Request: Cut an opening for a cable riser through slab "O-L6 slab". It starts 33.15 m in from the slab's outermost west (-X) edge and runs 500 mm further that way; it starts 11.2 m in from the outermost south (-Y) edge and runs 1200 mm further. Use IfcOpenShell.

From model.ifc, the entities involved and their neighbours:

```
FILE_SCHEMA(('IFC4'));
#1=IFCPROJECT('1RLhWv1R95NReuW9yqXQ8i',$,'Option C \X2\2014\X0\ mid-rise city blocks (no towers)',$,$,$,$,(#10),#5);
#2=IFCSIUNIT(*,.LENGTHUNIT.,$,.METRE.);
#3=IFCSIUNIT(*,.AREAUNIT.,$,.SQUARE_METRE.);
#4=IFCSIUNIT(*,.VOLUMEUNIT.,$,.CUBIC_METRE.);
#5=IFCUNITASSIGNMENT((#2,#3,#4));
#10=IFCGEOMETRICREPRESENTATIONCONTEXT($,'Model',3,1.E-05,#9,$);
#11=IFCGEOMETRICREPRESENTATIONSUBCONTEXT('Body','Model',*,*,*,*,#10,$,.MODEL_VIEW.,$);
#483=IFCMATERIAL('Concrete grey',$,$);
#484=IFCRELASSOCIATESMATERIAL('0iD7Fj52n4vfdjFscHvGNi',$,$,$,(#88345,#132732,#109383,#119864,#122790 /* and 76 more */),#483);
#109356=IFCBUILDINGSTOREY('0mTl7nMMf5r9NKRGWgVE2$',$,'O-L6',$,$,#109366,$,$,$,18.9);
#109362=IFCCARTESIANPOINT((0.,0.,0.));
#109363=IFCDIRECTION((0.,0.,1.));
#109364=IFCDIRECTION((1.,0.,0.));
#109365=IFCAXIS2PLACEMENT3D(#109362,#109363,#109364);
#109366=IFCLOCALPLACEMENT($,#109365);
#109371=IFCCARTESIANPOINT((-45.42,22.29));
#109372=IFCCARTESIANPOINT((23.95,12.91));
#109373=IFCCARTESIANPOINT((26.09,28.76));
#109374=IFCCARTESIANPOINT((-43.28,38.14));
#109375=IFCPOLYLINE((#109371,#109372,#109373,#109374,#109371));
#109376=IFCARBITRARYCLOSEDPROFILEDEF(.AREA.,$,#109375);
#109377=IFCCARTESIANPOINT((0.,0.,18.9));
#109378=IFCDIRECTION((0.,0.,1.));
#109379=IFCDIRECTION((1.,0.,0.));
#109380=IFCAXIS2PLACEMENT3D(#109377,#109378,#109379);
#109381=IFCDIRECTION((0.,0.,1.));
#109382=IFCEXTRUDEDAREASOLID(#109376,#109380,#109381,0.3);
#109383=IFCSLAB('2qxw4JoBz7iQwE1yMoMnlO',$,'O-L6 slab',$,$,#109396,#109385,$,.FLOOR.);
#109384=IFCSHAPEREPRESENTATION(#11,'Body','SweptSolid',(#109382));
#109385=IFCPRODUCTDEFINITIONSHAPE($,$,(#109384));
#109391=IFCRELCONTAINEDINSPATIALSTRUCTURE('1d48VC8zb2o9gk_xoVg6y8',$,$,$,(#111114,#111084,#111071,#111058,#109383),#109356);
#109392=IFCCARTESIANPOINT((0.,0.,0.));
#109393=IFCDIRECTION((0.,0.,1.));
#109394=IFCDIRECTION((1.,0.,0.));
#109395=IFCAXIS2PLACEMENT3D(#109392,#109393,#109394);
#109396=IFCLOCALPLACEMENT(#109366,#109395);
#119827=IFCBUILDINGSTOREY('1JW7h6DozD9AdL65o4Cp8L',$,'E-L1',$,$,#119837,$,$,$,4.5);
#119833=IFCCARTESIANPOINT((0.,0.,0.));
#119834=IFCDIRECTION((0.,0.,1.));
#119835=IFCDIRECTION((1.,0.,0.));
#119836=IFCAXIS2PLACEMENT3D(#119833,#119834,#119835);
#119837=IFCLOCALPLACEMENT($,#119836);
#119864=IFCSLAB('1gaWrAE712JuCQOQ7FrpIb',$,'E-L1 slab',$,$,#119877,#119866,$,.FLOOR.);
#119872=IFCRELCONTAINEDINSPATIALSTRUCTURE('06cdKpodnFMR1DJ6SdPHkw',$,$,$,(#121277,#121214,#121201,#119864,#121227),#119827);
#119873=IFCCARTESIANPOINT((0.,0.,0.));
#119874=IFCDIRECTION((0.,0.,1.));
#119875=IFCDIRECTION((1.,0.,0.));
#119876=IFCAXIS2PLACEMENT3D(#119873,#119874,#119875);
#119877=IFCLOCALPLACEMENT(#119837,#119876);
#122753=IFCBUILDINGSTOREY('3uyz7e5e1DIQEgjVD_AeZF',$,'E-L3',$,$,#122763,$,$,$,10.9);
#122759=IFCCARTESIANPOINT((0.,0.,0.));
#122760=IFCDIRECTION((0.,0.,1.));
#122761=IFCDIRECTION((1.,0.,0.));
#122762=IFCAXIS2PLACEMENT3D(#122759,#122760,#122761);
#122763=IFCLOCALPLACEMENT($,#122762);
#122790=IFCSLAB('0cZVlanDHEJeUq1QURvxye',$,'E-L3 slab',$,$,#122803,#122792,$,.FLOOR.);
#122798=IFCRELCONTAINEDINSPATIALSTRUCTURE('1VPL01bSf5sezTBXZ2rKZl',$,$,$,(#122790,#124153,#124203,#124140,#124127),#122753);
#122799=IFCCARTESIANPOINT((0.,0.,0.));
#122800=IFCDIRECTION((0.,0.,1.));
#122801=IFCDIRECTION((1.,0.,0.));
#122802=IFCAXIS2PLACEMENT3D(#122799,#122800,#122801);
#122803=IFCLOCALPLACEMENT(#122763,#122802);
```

```python
import numpy as np
import ifcopenshell
import ifcopenshell.api.feature
import ifcopenshell.api.geometry
import ifcopenshell.api.root
import ifcopenshell.geom
import ifcopenshell.util.placement
import ifcopenshell.util.representation
import ifcopenshell.util.shape
import ifcopenshell.util.unit

model = ifcopenshell.open("model.ifc")
unit_scale = ifcopenshell.util.unit.calculate_unit_scale(model)
settings = ifcopenshell.geom.settings()


def volume(element):
    """Net volume in cubic metres, openings subtracted."""
    shape = ifcopenshell.geom.create_shape(settings, element)
    return ifcopenshell.util.shape.get_volume(shape.geometry)


slab = model.by_guid("2qxw4JoBz7iQwE1yMoMnlO")
before = volume(slab)

# Extent in the slab's own axes, in metres. The edges named are its -X and -Y sides.
slab_shape = ifcopenshell.geom.create_shape(settings, slab)
vertices = ifcopenshell.util.shape.get_vertices(slab_shape.geometry)
x_min, y_min, bottom = vertices.min(axis=0)
top = vertices[:, 2].max()

opening = ifcopenshell.api.root.create_entity(model, ifc_class="IfcOpeningElement", name="Cable riser opening", predefined_type="OPENING")
context = ifcopenshell.util.representation.get_context(model, "Model", "Body", "MODEL_VIEW")
width, depth = 0.5, 1.2
outline = [(0.0, 0.0), (width, 0.0), (width, depth), (0.0, depth), (0.0, 0.0)]
# Overshoot both faces by 50 mm so the cut is clean.
shape = ifcopenshell.api.geometry.add_slab_representation(
    model, context=context, depth=top - bottom + 0.1, polyline=outline
)
ifcopenshell.api.geometry.assign_representation(model, product=opening, representation=shape)

matrix = ifcopenshell.util.placement.get_local_placement(slab.ObjectPlacement)
matrix[:, 3] = matrix @ np.append(np.array([x_min + 33.15, y_min + 11.2, bottom - 0.05]) / unit_scale, 1.0)
ifcopenshell.api.geometry.edit_object_placement(model, product=opening, matrix=matrix, is_si=False)
ifcopenshell.api.feature.add_feature(model, feature=opening, element=slab)

after = volume(slab)

print(f"slab volume {before:.3f} -> {after:.3f} m3")

model.write("model_v2.ifc")
```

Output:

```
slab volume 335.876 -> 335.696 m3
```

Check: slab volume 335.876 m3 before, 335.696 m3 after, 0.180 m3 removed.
